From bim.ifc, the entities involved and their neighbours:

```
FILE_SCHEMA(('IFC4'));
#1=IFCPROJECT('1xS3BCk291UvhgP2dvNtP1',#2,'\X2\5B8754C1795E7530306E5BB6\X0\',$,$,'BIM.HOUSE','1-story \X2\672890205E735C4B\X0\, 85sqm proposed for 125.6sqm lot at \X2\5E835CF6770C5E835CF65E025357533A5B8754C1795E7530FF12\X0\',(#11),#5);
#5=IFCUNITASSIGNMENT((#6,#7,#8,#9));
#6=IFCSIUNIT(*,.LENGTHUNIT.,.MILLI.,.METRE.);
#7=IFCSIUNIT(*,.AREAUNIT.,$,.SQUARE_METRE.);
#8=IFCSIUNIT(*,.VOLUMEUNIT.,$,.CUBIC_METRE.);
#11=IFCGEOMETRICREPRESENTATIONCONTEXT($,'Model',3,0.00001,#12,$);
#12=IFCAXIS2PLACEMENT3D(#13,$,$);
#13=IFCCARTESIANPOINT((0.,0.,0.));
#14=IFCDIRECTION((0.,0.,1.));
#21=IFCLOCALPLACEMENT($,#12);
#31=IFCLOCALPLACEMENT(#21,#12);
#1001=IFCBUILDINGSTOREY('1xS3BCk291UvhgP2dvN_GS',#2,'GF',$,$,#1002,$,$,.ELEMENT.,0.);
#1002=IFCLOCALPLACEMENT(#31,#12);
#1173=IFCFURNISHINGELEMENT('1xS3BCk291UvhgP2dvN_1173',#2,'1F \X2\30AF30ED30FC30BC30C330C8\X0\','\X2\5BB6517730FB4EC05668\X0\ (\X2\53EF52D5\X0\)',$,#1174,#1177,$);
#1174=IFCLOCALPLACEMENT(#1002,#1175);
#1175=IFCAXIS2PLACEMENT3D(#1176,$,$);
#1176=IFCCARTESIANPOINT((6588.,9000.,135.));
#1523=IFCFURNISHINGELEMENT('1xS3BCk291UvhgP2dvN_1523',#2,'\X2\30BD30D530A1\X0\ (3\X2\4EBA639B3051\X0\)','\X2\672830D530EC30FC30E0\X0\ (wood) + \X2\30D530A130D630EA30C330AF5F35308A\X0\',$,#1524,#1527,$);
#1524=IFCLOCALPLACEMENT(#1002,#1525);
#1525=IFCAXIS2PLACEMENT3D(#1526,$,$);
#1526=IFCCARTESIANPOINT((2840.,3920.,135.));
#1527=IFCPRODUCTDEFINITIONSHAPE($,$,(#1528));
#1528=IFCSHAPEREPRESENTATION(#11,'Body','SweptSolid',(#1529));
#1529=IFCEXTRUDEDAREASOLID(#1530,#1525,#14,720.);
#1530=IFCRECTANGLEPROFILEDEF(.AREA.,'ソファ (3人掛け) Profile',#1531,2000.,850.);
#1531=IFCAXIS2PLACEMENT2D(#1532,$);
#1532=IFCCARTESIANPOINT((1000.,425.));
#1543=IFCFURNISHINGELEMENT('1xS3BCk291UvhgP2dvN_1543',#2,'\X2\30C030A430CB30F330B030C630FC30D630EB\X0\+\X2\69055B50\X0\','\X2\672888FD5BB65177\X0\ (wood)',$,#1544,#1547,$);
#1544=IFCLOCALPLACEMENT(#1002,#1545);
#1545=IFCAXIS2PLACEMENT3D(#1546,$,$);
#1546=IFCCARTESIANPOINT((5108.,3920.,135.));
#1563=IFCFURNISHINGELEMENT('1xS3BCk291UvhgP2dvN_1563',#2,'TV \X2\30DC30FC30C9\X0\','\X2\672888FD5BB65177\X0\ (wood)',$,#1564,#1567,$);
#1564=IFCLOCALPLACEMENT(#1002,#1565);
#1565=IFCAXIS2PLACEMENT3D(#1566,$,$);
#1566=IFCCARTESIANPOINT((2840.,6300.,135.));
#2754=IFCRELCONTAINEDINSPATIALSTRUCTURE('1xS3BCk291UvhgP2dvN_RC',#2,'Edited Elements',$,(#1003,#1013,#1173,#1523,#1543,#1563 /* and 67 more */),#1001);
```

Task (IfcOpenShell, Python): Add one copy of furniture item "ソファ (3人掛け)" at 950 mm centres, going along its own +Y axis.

```python
import ifcopenshell
import ifcopenshell.api.geometry
import ifcopenshell.api.root
import ifcopenshell.util.element
import ifcopenshell.util.placement

model = ifcopenshell.open("bim.ifc")


def reuse_history(source, copy):
    """copy_class also copies each property set's owner history, people and application; keep the originals."""
    for rel in copy.IsDefinedBy:
        if rel.is_a("IfcRelDefinesByProperties") and (history := rel.RelatingPropertyDefinition.OwnerHistory):
            rel.RelatingPropertyDefinition.OwnerHistory = source.OwnerHistory
            ifcopenshell.util.element.remove_deep2(model, history)


source = model.by_guid("1xS3BCk291UvhgP2dvN_1523")
base = ifcopenshell.util.placement.get_local_placement(source.ObjectPlacement)
step = base[:3, 1] * 950.0

for i in range(1, 2):
    copy = ifcopenshell.api.root.copy_class(model, product=source)
    copy.Representation = ifcopenshell.util.element.copy_deep(
        model, source.Representation, exclude=["IfcGeometricRepresentationContext", "IfcRepresentationMap"]
    )
    reuse_history(source, copy)
    matrix = base.copy()
    matrix[:3, 3] += i * step
    print("added at", matrix[:3, 3].round(3) + 0.0)
    ifcopenshell.api.geometry.edit_object_placement(model, product=copy, matrix=matrix, is_si=False)

model.write("bim_updated.ifc")
```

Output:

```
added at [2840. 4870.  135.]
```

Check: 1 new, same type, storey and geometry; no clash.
